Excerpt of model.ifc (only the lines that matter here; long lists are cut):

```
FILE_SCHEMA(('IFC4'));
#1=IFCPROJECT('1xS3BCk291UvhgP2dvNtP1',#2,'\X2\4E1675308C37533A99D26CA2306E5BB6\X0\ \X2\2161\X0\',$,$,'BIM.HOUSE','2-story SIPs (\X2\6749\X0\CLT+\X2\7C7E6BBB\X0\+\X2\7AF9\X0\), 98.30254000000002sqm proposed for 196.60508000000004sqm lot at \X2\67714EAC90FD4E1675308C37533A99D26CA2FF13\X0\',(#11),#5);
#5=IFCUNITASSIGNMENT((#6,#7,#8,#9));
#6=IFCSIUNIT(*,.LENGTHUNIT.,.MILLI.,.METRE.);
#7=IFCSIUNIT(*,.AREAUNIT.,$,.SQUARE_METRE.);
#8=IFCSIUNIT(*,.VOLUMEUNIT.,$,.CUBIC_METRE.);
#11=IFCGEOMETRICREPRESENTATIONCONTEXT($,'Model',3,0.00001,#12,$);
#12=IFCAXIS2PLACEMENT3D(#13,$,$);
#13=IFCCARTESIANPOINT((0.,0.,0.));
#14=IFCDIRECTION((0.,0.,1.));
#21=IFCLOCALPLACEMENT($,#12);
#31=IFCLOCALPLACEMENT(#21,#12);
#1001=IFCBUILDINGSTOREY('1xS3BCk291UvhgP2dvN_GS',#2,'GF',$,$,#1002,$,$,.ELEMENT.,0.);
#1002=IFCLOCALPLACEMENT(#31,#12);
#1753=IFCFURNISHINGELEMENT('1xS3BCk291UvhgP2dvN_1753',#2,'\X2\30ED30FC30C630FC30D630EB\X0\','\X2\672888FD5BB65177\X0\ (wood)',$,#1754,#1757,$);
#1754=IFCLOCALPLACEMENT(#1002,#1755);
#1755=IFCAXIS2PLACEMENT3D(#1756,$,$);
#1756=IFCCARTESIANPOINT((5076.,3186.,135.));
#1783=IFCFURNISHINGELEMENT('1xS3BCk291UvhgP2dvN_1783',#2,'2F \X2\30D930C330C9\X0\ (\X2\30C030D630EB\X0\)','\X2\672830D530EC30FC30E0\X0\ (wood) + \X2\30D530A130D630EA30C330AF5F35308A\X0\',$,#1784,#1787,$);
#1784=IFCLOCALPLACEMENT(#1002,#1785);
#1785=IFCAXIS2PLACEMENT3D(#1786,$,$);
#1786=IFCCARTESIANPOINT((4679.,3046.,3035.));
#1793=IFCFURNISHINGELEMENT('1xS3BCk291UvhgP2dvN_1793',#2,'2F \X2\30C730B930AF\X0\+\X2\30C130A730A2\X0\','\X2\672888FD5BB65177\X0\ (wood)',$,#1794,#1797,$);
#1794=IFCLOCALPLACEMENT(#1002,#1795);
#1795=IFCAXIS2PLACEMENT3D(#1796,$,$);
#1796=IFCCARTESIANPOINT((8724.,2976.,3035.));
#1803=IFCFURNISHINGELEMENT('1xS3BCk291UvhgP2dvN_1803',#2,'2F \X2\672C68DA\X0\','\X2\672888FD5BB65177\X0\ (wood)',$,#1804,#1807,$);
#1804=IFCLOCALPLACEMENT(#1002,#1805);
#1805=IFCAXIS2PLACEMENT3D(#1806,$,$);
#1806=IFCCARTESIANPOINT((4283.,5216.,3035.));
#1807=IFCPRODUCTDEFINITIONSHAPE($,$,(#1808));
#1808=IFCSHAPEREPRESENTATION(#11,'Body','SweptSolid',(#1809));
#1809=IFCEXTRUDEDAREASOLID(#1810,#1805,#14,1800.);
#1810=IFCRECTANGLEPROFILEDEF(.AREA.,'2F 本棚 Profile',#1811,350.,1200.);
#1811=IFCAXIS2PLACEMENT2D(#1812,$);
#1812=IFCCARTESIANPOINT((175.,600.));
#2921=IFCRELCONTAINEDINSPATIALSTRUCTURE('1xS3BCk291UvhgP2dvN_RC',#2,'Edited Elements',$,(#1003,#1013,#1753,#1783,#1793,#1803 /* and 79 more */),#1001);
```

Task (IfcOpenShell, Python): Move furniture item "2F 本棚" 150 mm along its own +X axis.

```python
import ifcopenshell
import ifcopenshell.api.geometry
import ifcopenshell.util.placement

model = ifcopenshell.open("model.ifc")

item = model.by_guid("1xS3BCk291UvhgP2dvN_1803")
matrix = ifcopenshell.util.placement.get_local_placement(item.ObjectPlacement)
matrix[:3, 3] += matrix[:3, 0] * 150.0
ifcopenshell.api.geometry.edit_object_placement(model, product=item, matrix=matrix, is_si=False)

print(ifcopenshell.util.placement.get_local_placement(item.ObjectPlacement).round(3) + 0.0)

model.write("model_edited.ifc")
```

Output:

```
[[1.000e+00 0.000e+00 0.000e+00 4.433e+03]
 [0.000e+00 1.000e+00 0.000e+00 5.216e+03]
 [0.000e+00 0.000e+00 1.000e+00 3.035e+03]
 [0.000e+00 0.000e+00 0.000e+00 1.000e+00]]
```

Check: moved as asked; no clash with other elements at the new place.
